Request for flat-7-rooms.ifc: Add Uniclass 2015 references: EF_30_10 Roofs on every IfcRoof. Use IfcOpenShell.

First a look at what the model holds.

```python
import ifcopenshell

model = ifcopenshell.open("flat-7-rooms.ifc")
print(model.schema)
print("classifications:", [c.Name for c in model.by_type("IfcClassification")])
for ifc_class in ("IfcDoor", "IfcRoof", "IfcStair", "IfcWall", "IfcWindow"):
    print(ifc_class, len(model.by_type(ifc_class)))
```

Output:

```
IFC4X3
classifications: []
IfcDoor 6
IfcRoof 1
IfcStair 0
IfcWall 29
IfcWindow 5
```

```python
import ifcopenshell
import ifcopenshell.api.classification

model = ifcopenshell.open("flat-7-rooms.ifc")

system = ifcopenshell.api.classification.add_classification(model, classification="Uniclass 2015")

codes = {
    "IfcRoof": ("EF_30_10", "Roofs"),
}
for ifc_class, (code, name) in codes.items():
    products = model.by_type(ifc_class)
    ifcopenshell.api.classification.add_reference(
        model, products=products, classification=system, identification=code, name=name
    )
    print(code, len(products))

model.write("flat-7-rooms_rev.ifc")
```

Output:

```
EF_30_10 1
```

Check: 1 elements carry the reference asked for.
